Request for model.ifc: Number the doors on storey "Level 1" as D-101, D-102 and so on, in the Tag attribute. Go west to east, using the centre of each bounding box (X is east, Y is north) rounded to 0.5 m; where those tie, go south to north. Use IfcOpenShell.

First a look at what the model holds.

```python
import ifcopenshell
import ifcopenshell.util.element
import ifcopenshell.util.placement

model = ifcopenshell.open("model.ifc")
print(model.schema)
storey = next(s for s in model.by_type("IfcBuildingStorey") if s.Name == "Level 1")
doors = [e for e in ifcopenshell.util.element.get_decomposition(storey) if e.is_a("IfcDoor")]
for e in sorted(doors, key=lambda e: e.id()):
    origin = ifcopenshell.util.placement.get_local_placement(e.ObjectPlacement)[:3, 3]
    print(e.id(), e.Tag, e.Name, origin.round(2) + 0.0, sep=" | ")
```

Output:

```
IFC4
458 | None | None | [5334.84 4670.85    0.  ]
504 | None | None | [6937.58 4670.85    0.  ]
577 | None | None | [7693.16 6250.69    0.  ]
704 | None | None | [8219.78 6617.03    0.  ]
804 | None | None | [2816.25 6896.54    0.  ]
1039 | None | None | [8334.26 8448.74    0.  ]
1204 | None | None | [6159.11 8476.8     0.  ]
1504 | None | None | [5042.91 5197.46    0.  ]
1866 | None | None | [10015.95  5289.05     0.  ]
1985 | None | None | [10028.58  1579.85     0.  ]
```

```python
import ifcopenshell
import ifcopenshell.geom
import ifcopenshell.util.element
import ifcopenshell.util.shape

model = ifcopenshell.open("model.ifc")
settings = ifcopenshell.geom.settings()
settings.set("use-world-coords", True)


def centre(element):
    shape = ifcopenshell.geom.create_shape(settings, element)
    return ifcopenshell.util.shape.get_bbox_centroid(shape.geometry)


storey = next(s for s in model.by_type("IfcBuildingStorey") if s.Name == "Level 1")
doors = [e for e in ifcopenshell.util.element.get_decomposition(storey) if e.is_a("IfcDoor")]

# Insertion points can sit at a corner or the storey origin, so sort by the geometry (in metres).
centres = {e: centre(e) for e in doors}
doors.sort(key=lambda e: (round(centres[e][0] / 0.5), centres[e][1]))

for i, e in enumerate(doors, start=1):
    number = f"D-1{i:02d}"
    e.Tag = number
    print(e.id(), number)

model.write("model_rev.ifc")
```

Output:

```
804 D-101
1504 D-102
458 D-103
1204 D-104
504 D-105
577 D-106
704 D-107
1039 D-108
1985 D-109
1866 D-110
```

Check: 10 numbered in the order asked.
